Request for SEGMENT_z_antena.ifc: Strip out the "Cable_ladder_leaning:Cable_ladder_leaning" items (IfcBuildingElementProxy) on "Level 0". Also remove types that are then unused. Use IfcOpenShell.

First a look at what the model holds.

```python
import ifcopenshell
import ifcopenshell.util.element

model = ifcopenshell.open("SEGMENT_z_antena.ifc")
print(model.schema)
storey = next(s for s in model.by_type("IfcBuildingStorey") if s.Name == "Level 0")
proxies = [e for e in ifcopenshell.util.element.get_decomposition(storey) if e.is_a("IfcBuildingElementProxy")]
seen = {}
for e in proxies:
    element_type = ifcopenshell.util.element.get_type(e)
    name = element_type.Name if element_type not in (None, e) else None
    seen[name] = seen.get(name, 0) + 1
for name, count in sorted(seen.items(), key=str):
    print(count, "x", name)
```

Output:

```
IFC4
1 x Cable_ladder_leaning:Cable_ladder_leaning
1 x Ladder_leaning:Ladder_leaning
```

```python
import ifcopenshell
import ifcopenshell.api.root
import ifcopenshell.util.element

model = ifcopenshell.open("SEGMENT_z_antena.ifc")

storey = next(s for s in model.by_type("IfcBuildingStorey") if s.Name == "Level 0")
proxies = [e for e in ifcopenshell.util.element.get_decomposition(storey) if e.is_a("IfcBuildingElementProxy")]
targets = [e for e in proxies if (t := ifcopenshell.util.element.get_type(e)) not in (None, e) and t.Name == "Cable_ladder_leaning:Cable_ladder_leaning"]
types = {ifcopenshell.util.element.get_type(e) for e in targets} - {None, *targets}

for e in targets:
    ifcopenshell.api.root.remove_product(model, product=e)
print(len(targets), "removed")

unused = [t for t in types if not ifcopenshell.util.element.get_types(t)]
for t in unused:
    ifcopenshell.api.root.remove_product(model, product=t)
print(len(unused), "unused types removed")

model.write("SEGMENT_z_antena_updated.ifc")
```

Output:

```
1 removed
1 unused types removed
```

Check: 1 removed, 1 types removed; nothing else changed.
